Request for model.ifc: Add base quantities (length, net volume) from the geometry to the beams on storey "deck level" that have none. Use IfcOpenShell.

First a look at what the model holds.

```python
import ifcopenshell
import ifcopenshell.util.element
import ifcopenshell.util.unit

model = ifcopenshell.open("model.ifc")
print(model.schema)
for unit_type in ("LENGTHUNIT", "AREAUNIT", "VOLUMEUNIT"):
    print(unit_type, ifcopenshell.util.unit.calculate_unit_scale(model, unit_type))
storey = next(s for s in model.by_type("IfcBuildingStorey") if s.Name == "deck level")
beams = [e for e in ifcopenshell.util.element.get_decomposition(storey) if e.is_a("IfcBeam")]
for e in sorted(beams, key=lambda e: e.id()):
    print(e.id(), e.is_a(), e.Name, list(ifcopenshell.util.element.get_psets(e, qtos_only=True)), sep=" | ")
```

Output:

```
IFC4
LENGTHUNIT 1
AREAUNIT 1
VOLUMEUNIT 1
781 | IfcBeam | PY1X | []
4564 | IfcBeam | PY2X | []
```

```python
import ifcopenshell
import ifcopenshell.api.pset
import ifcopenshell.geom
import ifcopenshell.util.element
import ifcopenshell.util.shape
import ifcopenshell.util.unit

model = ifcopenshell.open("model.ifc")
unit_scale = ifcopenshell.util.unit.calculate_unit_scale(model)
volume_scale = ifcopenshell.util.unit.calculate_unit_scale(model, "VOLUMEUNIT")
settings = ifcopenshell.geom.settings()

storey = next(s for s in model.by_type("IfcBuildingStorey") if s.Name == "deck level")
beams = [e for e in ifcopenshell.util.element.get_decomposition(storey) if e.is_a("IfcBeam")]

for e in sorted(beams, key=lambda e: e.id()):
    if ifcopenshell.util.element.get_psets(e, qtos_only=True, should_inherit=False):
        continue
    # Geometry comes back in metres, in the element's own axes.
    shape = ifcopenshell.geom.create_shape(settings, e)
    values = {
        "Length": ifcopenshell.util.shape.get_max_xyz(shape.geometry) / unit_scale,
        "NetVolume": ifcopenshell.util.shape.get_volume(shape.geometry) / volume_scale,
    }
    qto = ifcopenshell.api.pset.add_qto(model, product=e, name="Qto_BeamBaseQuantities")
    ifcopenshell.api.pset.edit_qto(model, qto=qto, properties=values)
    print(e.id(), {k: round(v, 3) for k, v in values.items()})

model.write("model-out.ifc")
```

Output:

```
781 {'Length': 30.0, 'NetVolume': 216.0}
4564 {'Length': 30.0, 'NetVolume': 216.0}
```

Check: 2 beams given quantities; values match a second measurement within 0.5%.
